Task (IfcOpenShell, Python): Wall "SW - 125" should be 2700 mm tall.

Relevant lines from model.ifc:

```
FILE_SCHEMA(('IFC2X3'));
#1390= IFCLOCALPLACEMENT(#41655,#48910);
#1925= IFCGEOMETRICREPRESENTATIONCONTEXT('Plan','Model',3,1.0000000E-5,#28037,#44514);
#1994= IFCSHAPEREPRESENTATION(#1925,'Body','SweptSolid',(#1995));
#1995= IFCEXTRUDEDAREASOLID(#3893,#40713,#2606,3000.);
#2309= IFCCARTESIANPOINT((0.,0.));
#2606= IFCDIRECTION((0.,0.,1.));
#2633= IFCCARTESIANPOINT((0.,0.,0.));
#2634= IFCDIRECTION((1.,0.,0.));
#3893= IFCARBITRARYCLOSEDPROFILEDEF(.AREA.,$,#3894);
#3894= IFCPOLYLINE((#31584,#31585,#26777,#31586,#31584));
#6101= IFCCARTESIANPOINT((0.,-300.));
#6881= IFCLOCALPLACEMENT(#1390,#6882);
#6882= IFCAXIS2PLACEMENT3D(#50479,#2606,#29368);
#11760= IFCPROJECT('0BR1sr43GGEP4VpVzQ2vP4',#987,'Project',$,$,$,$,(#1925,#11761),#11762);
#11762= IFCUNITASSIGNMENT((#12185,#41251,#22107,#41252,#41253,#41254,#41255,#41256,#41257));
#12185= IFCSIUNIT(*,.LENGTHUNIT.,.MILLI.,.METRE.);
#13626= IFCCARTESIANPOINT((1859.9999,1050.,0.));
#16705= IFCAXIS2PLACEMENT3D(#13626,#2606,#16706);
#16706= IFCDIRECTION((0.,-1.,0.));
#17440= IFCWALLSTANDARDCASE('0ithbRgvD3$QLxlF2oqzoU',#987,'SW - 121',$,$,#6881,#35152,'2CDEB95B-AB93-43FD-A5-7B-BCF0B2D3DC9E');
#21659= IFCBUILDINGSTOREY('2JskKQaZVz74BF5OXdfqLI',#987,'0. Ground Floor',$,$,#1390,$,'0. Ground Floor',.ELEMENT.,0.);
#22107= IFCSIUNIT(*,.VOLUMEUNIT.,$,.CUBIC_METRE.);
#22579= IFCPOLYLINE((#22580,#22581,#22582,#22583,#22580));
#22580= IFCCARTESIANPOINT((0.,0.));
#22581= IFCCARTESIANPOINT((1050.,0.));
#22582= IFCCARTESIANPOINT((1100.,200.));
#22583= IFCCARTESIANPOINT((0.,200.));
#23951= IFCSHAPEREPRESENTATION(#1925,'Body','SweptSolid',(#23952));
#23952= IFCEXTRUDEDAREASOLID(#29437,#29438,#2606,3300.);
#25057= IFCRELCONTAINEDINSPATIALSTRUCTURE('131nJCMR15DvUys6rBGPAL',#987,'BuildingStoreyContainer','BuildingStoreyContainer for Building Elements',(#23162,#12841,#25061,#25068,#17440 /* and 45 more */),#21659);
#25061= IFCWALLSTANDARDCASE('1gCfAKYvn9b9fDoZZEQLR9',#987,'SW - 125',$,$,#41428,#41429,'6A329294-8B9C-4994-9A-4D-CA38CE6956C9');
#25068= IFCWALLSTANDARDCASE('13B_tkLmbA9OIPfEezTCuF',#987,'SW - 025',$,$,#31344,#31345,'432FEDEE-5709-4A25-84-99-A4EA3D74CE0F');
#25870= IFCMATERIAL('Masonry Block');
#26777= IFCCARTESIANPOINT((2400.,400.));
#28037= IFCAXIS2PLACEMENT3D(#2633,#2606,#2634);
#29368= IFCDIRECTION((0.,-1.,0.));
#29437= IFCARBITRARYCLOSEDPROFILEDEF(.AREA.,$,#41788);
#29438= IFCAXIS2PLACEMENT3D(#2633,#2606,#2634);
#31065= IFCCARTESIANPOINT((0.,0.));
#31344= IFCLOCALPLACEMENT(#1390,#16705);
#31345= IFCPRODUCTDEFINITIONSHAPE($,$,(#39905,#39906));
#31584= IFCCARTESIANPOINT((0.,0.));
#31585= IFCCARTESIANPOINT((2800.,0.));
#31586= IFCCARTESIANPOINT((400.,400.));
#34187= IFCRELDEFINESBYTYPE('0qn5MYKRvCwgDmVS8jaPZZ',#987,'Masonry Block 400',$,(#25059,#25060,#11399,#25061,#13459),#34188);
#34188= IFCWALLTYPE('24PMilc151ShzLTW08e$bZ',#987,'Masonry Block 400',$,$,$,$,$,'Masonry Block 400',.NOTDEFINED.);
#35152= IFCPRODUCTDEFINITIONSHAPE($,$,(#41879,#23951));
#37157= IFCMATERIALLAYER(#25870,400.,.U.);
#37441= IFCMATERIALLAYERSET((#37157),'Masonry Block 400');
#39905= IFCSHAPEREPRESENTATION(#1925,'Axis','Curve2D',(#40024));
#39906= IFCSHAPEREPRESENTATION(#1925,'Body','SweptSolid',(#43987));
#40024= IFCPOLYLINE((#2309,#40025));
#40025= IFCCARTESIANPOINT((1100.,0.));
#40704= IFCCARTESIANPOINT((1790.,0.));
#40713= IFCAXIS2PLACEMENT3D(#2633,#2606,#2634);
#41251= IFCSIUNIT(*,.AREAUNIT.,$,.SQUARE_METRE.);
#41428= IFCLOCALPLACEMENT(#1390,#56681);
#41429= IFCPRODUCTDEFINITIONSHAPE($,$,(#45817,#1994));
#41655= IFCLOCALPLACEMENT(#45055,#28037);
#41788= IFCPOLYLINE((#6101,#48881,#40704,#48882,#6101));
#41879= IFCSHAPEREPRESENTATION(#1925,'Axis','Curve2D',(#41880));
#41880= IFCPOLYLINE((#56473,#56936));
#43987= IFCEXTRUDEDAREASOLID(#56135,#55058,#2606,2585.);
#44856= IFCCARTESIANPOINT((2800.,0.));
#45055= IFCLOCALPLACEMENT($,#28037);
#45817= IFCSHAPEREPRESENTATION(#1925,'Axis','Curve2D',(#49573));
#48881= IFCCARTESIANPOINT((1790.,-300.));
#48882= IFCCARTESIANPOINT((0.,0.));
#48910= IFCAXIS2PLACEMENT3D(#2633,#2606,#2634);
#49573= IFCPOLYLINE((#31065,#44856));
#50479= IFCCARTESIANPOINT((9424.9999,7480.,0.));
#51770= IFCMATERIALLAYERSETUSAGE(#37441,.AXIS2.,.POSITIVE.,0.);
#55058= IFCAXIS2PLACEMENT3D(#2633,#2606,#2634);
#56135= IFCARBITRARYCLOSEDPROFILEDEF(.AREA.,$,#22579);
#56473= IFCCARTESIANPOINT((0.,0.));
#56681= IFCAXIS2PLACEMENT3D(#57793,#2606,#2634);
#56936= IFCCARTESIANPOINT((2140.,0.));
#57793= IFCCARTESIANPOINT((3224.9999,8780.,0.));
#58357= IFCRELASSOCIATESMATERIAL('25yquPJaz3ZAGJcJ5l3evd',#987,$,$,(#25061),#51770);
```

```python
import ifcopenshell
import ifcopenshell.geom
import ifcopenshell.util.shape

model = ifcopenshell.open("model.ifc")
settings = ifcopenshell.geom.settings()


def volume(element):
    """Net volume in cubic metres, openings subtracted."""
    shape = ifcopenshell.geom.create_shape(settings, element)
    return ifcopenshell.util.shape.get_volume(shape.geometry)


wall = model.by_guid("1gCfAKYvn9b9fDoZZEQLR9")
before = volume(wall)

body = next(r for r in wall.Representation.Representations if r.RepresentationIdentifier == "Body")
solid = body.Items[0]
old_height = solid.Depth
solid.Depth = 2700.0
after = volume(wall)

print(f"height {old_height:g} -> {solid.Depth:g}, volume {before:.3f} -> {after:.3f} m3")

model.write("model_edited.ifc")
```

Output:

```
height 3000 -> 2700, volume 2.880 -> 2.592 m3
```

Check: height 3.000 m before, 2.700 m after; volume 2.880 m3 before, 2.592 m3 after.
